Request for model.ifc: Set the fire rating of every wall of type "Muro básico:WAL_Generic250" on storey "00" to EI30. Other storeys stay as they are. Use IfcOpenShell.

First a look at what the model holds.

```python
import ifcopenshell
import ifcopenshell.util.element

model = ifcopenshell.open("model.ifc")
print(model.schema)
storey = next(s for s in model.by_type("IfcBuildingStorey") if s.Name == "00")
walls = [e for e in ifcopenshell.util.element.get_decomposition(storey) if e.is_a("IfcWall")]
seen = {}
for e in walls:
    element_type = ifcopenshell.util.element.get_type(e)
    key = (element_type.Name if element_type != e and element_type else None, ifcopenshell.util.element.get_pset(e, "Pset_WallCommon", "FireRating"))
    seen[key] = seen.get(key, 0) + 1
for (name, value), count in sorted(seen.items(), key=str):
    print(count, "x", name, "|", value)
```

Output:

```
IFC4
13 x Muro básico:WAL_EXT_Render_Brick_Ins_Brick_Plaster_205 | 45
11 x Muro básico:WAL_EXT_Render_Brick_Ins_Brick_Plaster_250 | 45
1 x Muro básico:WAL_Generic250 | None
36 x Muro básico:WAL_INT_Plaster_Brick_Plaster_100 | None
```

```python
import ifcopenshell
import ifcopenshell.api.pset
import ifcopenshell.util.element

model = ifcopenshell.open("model.ifc")

storey = next(s for s in model.by_type("IfcBuildingStorey") if s.Name == "00")
walls = [e for e in ifcopenshell.util.element.get_decomposition(storey) if e.is_a("IfcWall")]

count = 0
for e in walls:
    element_type = ifcopenshell.util.element.get_type(e)
    if element_type in (None, e) or element_type.Name != "Muro básico:WAL_Generic250":
        continue
    # add_pset returns the element's existing set when there is one.
    pset = ifcopenshell.api.pset.add_pset(model, product=e, name="Pset_WallCommon")
    ifcopenshell.api.pset.edit_pset(model, pset=pset, properties={"FireRating": "EI30"})
    count += 1

print(count, "walls updated")

model.write("model-out.ifc")
```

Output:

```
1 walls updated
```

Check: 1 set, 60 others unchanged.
